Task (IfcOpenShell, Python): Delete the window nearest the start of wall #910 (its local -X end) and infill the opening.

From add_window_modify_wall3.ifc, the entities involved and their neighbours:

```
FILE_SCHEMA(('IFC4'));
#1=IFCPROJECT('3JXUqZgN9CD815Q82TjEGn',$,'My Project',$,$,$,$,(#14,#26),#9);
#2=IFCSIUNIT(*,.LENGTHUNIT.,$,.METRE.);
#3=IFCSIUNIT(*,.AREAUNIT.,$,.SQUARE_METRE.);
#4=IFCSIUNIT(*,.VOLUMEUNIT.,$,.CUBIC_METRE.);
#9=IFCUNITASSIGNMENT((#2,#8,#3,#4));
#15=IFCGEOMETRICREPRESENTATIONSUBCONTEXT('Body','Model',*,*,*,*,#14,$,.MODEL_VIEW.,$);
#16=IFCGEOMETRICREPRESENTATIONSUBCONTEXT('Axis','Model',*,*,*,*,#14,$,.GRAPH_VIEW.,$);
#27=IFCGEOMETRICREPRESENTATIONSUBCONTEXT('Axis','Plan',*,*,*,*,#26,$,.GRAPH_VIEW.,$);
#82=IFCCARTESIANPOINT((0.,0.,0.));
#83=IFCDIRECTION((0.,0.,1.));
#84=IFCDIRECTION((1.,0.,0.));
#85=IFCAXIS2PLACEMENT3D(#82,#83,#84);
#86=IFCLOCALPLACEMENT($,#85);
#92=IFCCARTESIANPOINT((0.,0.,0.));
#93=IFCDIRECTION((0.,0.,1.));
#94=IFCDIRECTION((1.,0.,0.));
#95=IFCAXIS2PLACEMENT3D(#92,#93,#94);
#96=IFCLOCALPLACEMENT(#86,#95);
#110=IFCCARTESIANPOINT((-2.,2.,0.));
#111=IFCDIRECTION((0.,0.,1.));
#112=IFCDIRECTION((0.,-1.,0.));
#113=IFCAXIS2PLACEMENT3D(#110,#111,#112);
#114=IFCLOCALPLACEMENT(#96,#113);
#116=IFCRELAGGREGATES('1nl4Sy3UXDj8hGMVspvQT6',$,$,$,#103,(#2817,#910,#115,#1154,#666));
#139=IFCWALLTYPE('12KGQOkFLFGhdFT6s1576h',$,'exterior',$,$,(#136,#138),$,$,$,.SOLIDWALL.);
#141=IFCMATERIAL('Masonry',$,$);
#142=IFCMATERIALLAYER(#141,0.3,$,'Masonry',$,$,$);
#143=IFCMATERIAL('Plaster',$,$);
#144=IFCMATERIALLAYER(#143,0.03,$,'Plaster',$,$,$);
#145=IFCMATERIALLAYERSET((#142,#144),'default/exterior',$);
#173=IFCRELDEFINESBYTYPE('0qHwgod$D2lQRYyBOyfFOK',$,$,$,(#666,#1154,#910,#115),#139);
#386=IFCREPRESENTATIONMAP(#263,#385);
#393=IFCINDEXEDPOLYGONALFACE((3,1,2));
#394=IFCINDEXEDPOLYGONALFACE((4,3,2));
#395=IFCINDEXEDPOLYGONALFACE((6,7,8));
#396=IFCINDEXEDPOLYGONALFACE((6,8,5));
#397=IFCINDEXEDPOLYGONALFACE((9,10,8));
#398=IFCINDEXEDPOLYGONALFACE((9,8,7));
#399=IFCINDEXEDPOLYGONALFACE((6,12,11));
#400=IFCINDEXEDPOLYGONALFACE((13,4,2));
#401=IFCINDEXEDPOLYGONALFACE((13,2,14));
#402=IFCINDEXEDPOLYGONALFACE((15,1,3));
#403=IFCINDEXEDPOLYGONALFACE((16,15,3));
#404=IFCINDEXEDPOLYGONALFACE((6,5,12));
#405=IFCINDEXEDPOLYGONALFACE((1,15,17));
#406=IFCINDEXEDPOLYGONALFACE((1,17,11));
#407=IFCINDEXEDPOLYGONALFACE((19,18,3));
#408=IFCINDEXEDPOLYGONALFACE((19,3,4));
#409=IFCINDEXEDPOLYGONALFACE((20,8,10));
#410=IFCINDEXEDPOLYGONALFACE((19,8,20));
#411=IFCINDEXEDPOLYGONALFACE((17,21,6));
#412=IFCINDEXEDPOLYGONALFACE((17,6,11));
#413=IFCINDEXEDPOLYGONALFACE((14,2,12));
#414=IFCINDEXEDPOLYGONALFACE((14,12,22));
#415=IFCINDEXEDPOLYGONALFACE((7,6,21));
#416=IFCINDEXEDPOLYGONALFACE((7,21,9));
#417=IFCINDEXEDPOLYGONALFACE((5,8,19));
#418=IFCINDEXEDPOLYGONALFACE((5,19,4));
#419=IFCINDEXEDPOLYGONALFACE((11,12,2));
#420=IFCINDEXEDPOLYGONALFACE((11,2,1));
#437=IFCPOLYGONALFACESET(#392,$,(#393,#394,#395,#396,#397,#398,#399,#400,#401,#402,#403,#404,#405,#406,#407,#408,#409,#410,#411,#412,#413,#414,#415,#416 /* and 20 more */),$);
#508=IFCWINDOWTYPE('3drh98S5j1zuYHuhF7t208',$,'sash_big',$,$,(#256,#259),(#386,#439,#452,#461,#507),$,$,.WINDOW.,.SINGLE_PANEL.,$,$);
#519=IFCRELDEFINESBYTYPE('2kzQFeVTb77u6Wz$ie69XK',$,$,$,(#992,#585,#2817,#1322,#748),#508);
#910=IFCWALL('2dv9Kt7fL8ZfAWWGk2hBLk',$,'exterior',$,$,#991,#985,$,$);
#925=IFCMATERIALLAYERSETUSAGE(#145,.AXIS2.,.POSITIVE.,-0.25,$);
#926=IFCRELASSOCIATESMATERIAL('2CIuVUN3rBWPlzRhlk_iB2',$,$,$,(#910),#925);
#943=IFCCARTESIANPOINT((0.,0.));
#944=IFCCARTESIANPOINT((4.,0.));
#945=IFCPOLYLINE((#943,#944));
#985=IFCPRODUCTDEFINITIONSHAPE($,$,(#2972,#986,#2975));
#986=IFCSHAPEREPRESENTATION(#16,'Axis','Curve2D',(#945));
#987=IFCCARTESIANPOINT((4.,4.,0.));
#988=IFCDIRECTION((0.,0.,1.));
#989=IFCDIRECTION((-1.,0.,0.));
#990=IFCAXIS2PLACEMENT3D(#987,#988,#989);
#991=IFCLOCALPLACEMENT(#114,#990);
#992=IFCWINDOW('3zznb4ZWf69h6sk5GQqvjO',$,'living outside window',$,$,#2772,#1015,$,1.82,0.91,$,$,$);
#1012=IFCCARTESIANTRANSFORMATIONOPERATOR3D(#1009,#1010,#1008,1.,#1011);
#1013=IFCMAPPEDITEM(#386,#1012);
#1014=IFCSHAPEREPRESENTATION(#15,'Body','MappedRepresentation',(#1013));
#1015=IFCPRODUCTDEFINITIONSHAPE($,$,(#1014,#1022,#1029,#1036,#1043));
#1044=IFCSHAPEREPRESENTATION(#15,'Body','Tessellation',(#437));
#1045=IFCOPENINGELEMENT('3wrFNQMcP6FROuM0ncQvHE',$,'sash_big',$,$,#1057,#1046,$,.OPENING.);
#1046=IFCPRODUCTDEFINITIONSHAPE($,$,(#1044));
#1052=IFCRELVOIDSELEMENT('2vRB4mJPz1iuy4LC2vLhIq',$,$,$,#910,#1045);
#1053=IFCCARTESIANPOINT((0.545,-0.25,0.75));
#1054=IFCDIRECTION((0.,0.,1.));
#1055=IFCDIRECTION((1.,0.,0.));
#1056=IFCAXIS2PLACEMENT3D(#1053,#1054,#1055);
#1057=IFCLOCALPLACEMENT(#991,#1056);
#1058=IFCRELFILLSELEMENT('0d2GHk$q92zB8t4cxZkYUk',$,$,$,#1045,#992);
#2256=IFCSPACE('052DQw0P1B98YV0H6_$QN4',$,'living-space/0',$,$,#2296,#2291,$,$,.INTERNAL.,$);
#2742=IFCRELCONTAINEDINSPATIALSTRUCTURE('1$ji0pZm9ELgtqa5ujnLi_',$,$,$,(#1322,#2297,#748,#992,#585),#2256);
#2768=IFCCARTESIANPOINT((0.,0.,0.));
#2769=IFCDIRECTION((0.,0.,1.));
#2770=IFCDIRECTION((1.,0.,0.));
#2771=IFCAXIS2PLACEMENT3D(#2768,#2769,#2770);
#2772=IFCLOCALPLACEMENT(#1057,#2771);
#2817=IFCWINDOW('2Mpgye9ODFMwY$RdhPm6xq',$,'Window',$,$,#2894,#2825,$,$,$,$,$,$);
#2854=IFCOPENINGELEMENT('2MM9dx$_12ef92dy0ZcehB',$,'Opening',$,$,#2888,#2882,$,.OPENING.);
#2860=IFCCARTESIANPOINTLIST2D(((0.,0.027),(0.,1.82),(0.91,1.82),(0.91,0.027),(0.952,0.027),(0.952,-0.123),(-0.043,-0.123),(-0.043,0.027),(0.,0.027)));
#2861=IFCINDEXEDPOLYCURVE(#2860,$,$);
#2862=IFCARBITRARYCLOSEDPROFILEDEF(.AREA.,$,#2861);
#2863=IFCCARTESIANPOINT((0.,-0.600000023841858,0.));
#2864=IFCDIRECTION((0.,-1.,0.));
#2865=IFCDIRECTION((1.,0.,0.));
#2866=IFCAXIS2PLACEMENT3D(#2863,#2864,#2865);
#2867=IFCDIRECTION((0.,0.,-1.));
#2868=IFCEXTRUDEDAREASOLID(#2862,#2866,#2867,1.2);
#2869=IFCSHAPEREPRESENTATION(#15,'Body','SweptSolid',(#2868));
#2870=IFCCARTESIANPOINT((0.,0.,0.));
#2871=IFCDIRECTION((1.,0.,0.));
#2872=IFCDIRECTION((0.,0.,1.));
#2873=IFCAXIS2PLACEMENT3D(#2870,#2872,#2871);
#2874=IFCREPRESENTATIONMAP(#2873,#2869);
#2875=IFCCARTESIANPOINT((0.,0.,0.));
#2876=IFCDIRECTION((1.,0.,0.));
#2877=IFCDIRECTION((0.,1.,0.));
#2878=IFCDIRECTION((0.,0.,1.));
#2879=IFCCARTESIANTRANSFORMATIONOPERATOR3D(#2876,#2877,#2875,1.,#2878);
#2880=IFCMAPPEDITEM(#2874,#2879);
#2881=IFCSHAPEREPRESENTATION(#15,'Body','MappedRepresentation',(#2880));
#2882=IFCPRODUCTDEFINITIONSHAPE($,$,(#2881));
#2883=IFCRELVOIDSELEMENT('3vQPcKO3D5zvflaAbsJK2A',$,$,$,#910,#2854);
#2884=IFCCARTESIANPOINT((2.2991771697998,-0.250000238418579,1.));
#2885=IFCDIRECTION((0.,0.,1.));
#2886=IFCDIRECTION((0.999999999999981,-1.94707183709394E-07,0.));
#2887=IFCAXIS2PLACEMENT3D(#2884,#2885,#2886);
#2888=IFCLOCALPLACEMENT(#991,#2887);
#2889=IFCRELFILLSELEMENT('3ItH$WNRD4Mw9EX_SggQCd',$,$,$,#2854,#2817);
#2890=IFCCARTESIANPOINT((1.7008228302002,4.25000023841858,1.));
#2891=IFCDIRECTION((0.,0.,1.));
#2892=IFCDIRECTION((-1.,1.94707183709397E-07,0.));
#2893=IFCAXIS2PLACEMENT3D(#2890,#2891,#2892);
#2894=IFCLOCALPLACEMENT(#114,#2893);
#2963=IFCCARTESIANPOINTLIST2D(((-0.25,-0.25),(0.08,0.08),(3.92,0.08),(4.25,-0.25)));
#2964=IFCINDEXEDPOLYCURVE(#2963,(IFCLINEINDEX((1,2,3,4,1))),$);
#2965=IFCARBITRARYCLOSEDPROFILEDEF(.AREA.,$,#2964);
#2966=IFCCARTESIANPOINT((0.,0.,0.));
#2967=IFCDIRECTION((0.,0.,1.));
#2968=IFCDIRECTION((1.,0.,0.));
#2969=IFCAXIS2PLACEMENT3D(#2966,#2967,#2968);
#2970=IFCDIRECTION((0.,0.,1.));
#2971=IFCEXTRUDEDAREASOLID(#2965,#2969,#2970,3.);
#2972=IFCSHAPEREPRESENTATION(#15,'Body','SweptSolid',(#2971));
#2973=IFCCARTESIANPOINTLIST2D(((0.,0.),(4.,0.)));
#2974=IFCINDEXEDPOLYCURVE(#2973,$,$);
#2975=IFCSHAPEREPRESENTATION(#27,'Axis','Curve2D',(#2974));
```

```python
import ifcopenshell
import ifcopenshell.api.feature
import ifcopenshell.api.root
import ifcopenshell.geom
import ifcopenshell.util.shape

model = ifcopenshell.open("add_window_modify_wall3.ifc")
settings = ifcopenshell.geom.settings()


def volume(element):
    """Net volume in cubic metres, openings subtracted."""
    shape = ifcopenshell.geom.create_shape(settings, element)
    return ifcopenshell.util.shape.get_volume(shape.geometry)


window = model.by_guid("3zznb4ZWf69h6sk5GQqvjO")
opening = window.FillsVoids[0].RelatingOpeningElement
wall = opening.VoidsElements[0].RelatingBuildingElement
before = volume(wall)

ifcopenshell.api.root.remove_product(model, product=window)
ifcopenshell.api.feature.remove_feature(model, feature=opening)

after = volume(wall)

print(f"wall volume {before:.3f} -> {after:.3f} m3")

model.write("add_window_modify_wall3_edited.ifc")
```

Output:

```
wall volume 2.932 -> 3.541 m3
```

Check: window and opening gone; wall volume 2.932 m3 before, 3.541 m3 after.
